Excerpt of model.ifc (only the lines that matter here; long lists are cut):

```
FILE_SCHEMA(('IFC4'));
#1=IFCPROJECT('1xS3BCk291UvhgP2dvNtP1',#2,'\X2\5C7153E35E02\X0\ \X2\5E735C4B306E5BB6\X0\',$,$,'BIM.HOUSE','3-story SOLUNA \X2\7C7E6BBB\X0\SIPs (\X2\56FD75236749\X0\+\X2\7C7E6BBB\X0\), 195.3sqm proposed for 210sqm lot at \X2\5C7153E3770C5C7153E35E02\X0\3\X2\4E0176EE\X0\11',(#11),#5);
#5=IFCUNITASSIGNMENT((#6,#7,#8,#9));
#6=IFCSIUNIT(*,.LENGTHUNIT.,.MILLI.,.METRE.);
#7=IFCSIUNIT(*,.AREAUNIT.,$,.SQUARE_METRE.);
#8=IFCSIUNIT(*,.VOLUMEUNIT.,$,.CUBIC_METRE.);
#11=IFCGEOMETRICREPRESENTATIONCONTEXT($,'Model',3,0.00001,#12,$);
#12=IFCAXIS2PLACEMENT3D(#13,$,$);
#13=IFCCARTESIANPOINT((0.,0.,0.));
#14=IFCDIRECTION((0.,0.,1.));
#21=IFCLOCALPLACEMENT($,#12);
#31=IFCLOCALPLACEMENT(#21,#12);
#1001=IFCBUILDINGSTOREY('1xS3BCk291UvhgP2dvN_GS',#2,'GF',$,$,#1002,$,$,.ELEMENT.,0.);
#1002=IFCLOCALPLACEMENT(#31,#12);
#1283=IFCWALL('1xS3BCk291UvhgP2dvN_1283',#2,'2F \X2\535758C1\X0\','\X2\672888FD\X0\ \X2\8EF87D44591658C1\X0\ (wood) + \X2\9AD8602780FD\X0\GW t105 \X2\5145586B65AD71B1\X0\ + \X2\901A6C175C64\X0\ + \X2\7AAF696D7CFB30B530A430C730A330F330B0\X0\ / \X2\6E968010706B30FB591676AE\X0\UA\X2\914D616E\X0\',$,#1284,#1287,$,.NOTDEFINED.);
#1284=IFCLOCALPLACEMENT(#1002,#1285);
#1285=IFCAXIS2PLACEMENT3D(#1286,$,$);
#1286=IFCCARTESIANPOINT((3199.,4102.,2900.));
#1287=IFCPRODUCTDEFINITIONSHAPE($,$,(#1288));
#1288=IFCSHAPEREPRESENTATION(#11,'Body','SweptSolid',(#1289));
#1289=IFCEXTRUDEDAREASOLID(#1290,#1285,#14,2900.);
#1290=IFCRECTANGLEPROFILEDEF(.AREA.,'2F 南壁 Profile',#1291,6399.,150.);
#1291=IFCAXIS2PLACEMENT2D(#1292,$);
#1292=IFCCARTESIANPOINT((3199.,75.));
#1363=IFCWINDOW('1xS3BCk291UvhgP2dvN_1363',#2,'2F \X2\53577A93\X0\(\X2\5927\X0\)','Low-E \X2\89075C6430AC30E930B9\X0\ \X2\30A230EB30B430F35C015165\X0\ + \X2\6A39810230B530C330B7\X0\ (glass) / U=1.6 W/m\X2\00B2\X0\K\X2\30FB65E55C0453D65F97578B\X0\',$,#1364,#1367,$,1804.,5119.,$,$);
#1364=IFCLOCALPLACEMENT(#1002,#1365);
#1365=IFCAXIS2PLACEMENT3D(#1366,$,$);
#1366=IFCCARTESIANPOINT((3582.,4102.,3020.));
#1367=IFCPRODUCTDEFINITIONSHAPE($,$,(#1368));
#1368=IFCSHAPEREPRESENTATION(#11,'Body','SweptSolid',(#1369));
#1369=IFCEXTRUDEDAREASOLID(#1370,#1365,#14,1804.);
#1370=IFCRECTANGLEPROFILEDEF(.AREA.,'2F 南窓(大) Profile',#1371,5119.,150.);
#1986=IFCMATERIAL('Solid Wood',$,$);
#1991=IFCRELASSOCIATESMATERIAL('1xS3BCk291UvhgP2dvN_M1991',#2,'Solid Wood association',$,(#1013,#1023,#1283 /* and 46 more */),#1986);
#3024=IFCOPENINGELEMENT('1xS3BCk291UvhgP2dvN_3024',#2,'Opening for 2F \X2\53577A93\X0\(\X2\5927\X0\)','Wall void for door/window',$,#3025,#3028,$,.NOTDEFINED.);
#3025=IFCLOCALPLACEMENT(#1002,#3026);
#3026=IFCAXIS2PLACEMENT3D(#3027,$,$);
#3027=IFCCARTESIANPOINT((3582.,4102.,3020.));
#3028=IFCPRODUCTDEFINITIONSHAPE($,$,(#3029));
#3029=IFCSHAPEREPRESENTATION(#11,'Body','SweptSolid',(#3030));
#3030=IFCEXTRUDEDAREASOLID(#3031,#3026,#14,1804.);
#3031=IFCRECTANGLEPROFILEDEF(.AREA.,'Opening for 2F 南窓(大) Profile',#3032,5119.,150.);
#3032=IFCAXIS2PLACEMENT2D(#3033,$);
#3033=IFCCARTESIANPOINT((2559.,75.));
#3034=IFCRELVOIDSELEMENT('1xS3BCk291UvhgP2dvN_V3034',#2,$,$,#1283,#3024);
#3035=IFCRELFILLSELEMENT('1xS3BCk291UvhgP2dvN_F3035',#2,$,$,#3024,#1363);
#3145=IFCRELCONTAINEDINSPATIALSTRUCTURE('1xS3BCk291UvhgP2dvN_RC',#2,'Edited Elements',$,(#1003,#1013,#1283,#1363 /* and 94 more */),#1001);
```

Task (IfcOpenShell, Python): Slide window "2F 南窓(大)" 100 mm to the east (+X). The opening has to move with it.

```python
import ifcopenshell
import ifcopenshell.api.geometry
import ifcopenshell.util.placement
import ifcopenshell.util.unit

model = ifcopenshell.open("model.ifc")
unit_scale = ifcopenshell.util.unit.calculate_unit_scale(model)

window = model.by_guid("1xS3BCk291UvhgP2dvN_1363")
opening = window.FillsVoids[0].RelatingOpeningElement
wall = opening.VoidsElements[0].RelatingBuildingElement

wall_matrix = ifcopenshell.util.placement.get_local_placement(wall.ObjectPlacement)
shift = wall_matrix[:3, 0] * 0.1 / unit_scale
before = ifcopenshell.util.placement.get_local_placement(window.ObjectPlacement)[:3, 3].copy()

# The window is not placed relative to its opening, so move both.
for product in (opening, window):
    matrix = ifcopenshell.util.placement.get_local_placement(product.ObjectPlacement)
    matrix[:3, 3] += shift
    ifcopenshell.api.geometry.edit_object_placement(model, product=product, matrix=matrix, is_si=False)

after = ifcopenshell.util.placement.get_local_placement(window.ObjectPlacement)[:3, 3]
print("window moved by", (after - before).round(3) + 0.0)

model.write("model_v2.ifc")
```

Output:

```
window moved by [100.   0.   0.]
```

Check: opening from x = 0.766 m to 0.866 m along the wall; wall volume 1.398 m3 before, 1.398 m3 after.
